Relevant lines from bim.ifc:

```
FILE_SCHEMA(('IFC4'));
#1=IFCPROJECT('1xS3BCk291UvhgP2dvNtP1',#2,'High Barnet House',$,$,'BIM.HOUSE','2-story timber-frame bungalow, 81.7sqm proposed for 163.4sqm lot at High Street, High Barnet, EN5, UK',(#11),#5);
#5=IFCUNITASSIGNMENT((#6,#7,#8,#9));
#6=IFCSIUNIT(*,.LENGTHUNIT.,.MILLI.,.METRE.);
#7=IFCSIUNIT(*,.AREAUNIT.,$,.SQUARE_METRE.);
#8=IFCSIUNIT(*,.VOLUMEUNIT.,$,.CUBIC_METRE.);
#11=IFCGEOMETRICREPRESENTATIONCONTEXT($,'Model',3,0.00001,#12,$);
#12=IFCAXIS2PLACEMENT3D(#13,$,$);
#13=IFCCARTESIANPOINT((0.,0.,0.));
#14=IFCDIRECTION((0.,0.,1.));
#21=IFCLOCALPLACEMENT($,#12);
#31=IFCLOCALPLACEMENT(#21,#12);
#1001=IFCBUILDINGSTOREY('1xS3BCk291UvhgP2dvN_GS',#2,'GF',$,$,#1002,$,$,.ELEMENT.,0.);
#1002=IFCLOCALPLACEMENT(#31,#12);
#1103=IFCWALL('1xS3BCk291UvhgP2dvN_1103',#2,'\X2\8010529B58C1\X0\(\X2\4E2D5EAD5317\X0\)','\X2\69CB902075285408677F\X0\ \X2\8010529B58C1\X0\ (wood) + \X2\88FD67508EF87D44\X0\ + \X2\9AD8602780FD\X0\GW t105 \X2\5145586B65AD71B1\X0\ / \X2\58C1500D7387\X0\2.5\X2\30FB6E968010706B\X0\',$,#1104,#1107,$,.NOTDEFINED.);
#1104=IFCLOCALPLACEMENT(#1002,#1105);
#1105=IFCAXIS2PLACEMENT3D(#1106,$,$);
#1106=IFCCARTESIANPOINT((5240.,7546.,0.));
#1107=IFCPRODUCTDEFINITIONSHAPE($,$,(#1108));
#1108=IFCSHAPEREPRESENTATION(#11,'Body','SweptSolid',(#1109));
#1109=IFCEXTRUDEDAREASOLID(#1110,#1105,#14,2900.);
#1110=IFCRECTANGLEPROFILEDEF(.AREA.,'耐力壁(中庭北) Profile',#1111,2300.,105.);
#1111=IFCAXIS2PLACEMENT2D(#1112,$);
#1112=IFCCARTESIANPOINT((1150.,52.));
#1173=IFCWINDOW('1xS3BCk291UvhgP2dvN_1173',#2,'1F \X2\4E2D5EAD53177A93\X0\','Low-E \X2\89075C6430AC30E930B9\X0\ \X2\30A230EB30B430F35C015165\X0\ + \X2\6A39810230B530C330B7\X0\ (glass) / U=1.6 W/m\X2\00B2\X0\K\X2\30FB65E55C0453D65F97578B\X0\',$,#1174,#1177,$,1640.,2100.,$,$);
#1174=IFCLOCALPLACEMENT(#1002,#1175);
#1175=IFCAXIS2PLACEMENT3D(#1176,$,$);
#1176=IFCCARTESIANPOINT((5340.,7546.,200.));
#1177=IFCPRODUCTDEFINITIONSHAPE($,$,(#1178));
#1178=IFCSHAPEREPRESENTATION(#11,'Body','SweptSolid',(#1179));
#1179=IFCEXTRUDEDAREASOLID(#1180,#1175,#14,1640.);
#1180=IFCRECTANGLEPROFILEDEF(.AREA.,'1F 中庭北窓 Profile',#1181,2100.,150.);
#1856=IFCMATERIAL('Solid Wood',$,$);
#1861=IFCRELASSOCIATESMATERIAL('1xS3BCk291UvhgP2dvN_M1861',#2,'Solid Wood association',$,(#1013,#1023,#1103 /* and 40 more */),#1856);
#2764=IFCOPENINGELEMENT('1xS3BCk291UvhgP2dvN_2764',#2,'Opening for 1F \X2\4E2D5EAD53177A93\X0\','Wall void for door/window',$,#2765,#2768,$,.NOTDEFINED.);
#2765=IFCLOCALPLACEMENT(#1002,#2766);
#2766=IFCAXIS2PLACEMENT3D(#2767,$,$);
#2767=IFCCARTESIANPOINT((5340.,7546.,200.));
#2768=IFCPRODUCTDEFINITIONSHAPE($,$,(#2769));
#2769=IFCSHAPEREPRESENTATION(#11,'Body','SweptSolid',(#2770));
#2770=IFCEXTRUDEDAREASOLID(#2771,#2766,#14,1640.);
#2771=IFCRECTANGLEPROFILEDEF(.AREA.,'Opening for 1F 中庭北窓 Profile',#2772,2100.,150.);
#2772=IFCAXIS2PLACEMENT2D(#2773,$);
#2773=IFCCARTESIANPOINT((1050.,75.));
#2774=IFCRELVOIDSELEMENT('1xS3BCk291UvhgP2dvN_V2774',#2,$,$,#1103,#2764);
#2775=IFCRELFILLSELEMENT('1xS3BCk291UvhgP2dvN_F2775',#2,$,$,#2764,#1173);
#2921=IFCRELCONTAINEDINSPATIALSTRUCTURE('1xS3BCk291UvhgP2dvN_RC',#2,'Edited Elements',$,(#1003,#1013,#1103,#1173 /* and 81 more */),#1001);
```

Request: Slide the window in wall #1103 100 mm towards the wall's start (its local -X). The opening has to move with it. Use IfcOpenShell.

```python
import ifcopenshell
import ifcopenshell.api.geometry
import ifcopenshell.util.placement

model = ifcopenshell.open("bim.ifc")

window = model.by_guid("1xS3BCk291UvhgP2dvN_1173")
opening = window.FillsVoids[0].RelatingOpeningElement
wall = opening.VoidsElements[0].RelatingBuildingElement

wall_matrix = ifcopenshell.util.placement.get_local_placement(wall.ObjectPlacement)
shift = wall_matrix[:3, 0] * -100.0
before = ifcopenshell.util.placement.get_local_placement(window.ObjectPlacement)[:3, 3].copy()

# The window is not placed relative to its opening, so move both.
for product in (opening, window):
    matrix = ifcopenshell.util.placement.get_local_placement(product.ObjectPlacement)
    matrix[:3, 3] += shift
    ifcopenshell.api.geometry.edit_object_placement(model, product=product, matrix=matrix, is_si=False)

after = ifcopenshell.util.placement.get_local_placement(window.ObjectPlacement)[:3, 3]
print("window moved by", (after - before).round(3) + 0.0)

model.write("bim_updated.ifc")
```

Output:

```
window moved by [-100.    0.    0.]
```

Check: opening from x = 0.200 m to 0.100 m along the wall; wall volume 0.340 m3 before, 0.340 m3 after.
